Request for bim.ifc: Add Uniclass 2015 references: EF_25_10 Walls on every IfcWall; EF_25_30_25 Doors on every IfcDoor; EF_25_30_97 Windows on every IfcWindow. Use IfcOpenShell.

First a look at what the model holds.

```python
import ifcopenshell

model = ifcopenshell.open("bim.ifc")
print(model.schema)
print("classifications:", [c.Name for c in model.by_type("IfcClassification")])
for ifc_class in ("IfcDoor", "IfcRoof", "IfcStair", "IfcWall", "IfcWindow"):
    print(ifc_class, len(model.by_type(ifc_class)))
```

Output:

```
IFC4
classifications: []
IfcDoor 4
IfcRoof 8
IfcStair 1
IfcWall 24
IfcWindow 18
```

```python
import ifcopenshell
import ifcopenshell.api.classification

model = ifcopenshell.open("bim.ifc")

system = ifcopenshell.api.classification.add_classification(model, classification="Uniclass 2015")

codes = {
    "IfcWall": ("EF_25_10", "Walls"),
    "IfcDoor": ("EF_25_30_25", "Doors"),
    "IfcWindow": ("EF_25_30_97", "Windows"),
}
for ifc_class, (code, name) in codes.items():
    products = model.by_type(ifc_class)
    ifcopenshell.api.classification.add_reference(
        model, products=products, classification=system, identification=code, name=name
    )
    print(code, len(products))

model.write("bim_v2.ifc")
```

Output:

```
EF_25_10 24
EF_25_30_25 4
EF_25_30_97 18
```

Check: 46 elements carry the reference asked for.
